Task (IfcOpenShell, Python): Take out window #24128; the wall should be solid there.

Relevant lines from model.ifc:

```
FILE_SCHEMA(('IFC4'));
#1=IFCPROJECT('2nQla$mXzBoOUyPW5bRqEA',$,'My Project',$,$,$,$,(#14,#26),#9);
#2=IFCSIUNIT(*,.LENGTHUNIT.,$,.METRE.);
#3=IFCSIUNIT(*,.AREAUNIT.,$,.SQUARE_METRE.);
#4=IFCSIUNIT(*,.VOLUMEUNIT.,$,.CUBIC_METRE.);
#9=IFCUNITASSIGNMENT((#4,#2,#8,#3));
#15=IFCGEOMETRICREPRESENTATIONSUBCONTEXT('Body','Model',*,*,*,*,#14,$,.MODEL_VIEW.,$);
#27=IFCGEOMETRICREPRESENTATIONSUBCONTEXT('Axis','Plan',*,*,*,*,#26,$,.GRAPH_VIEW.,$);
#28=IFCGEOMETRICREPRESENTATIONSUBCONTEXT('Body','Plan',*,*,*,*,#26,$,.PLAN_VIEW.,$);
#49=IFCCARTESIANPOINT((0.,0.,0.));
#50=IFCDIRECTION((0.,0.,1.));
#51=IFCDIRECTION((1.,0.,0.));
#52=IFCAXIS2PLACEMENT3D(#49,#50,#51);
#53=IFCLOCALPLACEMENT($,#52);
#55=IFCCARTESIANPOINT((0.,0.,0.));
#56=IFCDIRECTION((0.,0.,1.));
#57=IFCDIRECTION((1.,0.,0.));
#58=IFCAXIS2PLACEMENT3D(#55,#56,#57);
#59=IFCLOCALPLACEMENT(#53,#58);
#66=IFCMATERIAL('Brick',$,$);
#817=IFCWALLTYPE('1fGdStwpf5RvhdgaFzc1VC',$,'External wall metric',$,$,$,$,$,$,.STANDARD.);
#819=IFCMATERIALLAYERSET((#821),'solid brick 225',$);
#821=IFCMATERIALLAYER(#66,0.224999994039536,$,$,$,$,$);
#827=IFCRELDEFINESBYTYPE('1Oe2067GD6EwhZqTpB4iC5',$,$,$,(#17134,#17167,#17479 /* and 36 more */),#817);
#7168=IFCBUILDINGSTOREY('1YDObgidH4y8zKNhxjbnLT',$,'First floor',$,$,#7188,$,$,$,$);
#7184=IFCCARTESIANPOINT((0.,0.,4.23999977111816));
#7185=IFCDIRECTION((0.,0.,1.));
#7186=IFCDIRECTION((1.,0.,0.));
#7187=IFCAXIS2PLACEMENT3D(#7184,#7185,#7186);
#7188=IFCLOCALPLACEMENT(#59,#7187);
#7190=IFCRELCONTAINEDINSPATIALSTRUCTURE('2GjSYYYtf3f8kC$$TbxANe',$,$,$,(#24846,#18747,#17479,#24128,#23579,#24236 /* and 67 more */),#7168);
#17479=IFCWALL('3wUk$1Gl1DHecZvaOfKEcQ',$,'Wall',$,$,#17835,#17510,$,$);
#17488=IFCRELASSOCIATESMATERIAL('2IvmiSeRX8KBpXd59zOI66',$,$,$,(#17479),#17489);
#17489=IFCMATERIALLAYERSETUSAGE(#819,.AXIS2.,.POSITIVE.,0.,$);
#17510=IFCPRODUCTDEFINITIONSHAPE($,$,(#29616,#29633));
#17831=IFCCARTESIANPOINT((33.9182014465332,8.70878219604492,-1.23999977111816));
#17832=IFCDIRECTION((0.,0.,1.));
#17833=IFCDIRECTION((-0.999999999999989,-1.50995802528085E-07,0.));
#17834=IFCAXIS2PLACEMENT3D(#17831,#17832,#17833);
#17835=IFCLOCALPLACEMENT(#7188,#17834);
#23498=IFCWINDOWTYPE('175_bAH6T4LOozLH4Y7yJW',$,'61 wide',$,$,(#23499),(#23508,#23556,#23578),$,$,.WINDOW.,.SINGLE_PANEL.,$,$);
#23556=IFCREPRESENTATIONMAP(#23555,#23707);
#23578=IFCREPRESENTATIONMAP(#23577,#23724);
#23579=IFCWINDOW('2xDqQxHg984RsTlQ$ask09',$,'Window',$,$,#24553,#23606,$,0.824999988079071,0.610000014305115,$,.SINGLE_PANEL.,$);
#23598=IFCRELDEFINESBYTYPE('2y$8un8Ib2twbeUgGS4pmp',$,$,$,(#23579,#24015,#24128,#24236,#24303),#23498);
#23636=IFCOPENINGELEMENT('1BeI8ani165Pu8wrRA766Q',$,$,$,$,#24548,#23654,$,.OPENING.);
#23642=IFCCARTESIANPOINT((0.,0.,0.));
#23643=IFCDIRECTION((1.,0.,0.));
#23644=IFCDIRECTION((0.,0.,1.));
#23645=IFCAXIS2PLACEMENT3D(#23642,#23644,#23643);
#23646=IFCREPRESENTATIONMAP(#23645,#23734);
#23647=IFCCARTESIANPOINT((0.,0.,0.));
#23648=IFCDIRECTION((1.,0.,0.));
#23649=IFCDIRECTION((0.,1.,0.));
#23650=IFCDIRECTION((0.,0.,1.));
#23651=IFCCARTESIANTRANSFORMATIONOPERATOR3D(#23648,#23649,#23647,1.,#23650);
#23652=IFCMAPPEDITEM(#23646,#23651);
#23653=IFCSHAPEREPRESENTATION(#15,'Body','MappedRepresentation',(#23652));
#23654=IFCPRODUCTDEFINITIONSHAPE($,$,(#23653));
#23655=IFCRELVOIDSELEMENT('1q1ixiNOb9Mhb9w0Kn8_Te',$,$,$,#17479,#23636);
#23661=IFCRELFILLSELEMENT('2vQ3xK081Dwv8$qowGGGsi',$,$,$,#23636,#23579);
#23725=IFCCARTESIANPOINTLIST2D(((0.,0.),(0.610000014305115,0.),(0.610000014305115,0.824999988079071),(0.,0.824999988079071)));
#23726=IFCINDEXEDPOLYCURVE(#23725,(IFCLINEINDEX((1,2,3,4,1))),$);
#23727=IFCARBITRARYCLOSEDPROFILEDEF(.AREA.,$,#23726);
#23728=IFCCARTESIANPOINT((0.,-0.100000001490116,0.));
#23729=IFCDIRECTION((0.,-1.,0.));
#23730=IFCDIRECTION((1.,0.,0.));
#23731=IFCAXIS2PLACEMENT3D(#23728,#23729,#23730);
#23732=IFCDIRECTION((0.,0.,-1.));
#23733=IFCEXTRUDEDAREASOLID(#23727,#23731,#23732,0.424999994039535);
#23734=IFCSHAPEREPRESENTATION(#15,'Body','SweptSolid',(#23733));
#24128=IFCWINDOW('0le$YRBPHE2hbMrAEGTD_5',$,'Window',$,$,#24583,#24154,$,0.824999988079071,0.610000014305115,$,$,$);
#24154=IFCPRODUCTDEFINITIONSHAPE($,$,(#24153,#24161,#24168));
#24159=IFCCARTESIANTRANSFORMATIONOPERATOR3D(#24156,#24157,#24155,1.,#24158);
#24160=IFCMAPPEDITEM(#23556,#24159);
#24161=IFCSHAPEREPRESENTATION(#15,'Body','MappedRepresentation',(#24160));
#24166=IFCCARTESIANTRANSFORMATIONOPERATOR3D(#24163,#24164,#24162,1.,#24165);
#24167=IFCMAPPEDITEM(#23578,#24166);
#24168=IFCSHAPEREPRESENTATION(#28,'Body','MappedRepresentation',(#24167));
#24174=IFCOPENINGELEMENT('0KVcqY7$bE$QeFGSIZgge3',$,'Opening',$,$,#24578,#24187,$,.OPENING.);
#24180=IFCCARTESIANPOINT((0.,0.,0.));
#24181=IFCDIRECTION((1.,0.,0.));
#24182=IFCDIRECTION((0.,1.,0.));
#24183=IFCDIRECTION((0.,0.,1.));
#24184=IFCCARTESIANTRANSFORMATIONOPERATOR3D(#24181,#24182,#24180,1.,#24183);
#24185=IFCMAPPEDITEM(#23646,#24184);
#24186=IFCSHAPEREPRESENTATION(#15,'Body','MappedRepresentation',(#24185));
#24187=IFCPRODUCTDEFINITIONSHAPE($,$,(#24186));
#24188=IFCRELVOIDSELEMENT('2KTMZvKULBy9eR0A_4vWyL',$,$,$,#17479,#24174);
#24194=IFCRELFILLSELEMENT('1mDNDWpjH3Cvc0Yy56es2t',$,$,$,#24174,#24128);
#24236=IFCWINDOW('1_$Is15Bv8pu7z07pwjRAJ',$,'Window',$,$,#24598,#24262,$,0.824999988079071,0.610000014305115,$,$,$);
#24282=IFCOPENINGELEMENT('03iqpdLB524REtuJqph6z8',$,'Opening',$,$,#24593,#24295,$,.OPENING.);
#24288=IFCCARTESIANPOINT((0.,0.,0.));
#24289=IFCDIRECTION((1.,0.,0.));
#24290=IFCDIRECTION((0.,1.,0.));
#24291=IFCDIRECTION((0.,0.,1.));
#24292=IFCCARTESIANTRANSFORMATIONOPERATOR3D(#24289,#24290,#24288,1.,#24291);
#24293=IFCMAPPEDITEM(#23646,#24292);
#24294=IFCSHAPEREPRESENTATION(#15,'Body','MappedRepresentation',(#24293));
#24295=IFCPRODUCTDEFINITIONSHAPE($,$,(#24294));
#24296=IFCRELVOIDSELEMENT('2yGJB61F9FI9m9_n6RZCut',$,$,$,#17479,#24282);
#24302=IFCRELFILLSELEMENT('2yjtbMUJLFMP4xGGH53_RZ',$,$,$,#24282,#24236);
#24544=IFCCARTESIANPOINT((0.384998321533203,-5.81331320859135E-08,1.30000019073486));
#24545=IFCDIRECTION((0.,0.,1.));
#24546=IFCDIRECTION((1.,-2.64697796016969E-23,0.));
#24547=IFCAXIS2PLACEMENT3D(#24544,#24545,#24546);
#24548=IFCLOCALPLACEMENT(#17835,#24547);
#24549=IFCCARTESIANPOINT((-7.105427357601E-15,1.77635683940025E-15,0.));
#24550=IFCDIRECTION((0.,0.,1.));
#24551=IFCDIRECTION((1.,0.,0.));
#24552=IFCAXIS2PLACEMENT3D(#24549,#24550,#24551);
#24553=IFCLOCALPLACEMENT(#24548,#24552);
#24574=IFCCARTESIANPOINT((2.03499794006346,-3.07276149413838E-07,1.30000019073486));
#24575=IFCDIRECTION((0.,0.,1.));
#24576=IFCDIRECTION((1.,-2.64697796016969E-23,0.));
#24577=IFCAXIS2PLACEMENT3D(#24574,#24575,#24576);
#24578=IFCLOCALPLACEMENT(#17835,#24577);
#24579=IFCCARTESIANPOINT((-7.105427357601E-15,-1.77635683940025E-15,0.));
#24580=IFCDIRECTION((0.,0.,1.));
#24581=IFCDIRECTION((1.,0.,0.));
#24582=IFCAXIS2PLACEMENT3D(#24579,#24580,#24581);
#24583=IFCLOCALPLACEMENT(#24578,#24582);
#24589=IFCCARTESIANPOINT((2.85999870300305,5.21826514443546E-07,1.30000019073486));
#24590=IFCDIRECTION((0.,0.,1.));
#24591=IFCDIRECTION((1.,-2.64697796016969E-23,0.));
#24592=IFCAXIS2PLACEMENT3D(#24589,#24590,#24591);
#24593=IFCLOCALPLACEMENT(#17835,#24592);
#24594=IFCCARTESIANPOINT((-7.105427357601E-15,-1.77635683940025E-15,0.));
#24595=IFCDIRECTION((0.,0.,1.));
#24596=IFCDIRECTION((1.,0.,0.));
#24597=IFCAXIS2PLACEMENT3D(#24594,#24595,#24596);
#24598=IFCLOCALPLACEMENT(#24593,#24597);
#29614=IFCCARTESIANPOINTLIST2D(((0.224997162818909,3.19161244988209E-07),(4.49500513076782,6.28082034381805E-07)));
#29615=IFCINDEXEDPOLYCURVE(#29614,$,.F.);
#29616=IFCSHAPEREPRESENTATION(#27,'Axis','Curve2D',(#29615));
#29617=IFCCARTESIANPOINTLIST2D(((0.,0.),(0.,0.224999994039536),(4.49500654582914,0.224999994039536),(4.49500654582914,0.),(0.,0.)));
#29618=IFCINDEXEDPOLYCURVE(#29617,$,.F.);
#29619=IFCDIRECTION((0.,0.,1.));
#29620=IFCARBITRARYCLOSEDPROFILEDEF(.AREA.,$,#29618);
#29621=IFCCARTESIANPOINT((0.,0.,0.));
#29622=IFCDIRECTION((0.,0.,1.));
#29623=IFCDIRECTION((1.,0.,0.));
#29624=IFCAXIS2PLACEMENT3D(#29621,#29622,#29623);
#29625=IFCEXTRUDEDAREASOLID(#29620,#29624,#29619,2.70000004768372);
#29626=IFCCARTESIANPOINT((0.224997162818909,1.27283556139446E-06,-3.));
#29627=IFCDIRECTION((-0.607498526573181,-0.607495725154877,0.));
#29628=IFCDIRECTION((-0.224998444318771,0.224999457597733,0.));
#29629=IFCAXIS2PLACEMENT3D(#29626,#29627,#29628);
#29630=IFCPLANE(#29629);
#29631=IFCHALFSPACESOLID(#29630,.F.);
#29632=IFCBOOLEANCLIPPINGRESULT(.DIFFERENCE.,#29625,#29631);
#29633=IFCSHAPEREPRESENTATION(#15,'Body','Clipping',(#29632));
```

```python
import ifcopenshell
import ifcopenshell.api.feature
import ifcopenshell.api.root
import ifcopenshell.geom
import ifcopenshell.util.shape

model = ifcopenshell.open("model.ifc")
settings = ifcopenshell.geom.settings()


def volume(element):
    """Net volume in cubic metres, openings subtracted."""
    shape = ifcopenshell.geom.create_shape(settings, element)
    return ifcopenshell.util.shape.get_volume(shape.geometry)


window = model.by_guid("0le$YRBPHE2hbMrAEGTD_5")
opening = window.FillsVoids[0].RelatingOpeningElement
wall = opening.VoidsElements[0].RelatingBuildingElement
before = volume(wall)

ifcopenshell.api.root.remove_product(model, product=window)
ifcopenshell.api.feature.remove_feature(model, feature=opening)

after = volume(wall)

print(f"wall volume {before:.3f} -> {after:.3f} m3")

model.write("model_updated.ifc")
```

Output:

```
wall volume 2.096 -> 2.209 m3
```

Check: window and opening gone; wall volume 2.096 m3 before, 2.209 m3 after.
